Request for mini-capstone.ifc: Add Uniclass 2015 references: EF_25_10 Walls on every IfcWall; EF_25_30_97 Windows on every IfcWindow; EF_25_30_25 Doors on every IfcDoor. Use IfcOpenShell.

First a look at what the model holds.

```python
import ifcopenshell

model = ifcopenshell.open("mini-capstone.ifc")
print(model.schema)
print("classifications:", [c.Name for c in model.by_type("IfcClassification")])
for ifc_class in ("IfcDoor", "IfcRoof", "IfcStair", "IfcWall", "IfcWindow"):
    print(ifc_class, len(model.by_type(ifc_class)))
```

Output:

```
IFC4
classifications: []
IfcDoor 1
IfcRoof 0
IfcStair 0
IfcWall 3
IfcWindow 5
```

```python
import ifcopenshell
import ifcopenshell.api.classification

model = ifcopenshell.open("mini-capstone.ifc")

system = ifcopenshell.api.classification.add_classification(model, classification="Uniclass 2015")

codes = {
    "IfcWall": ("EF_25_10", "Walls"),
    "IfcWindow": ("EF_25_30_97", "Windows"),
    "IfcDoor": ("EF_25_30_25", "Doors"),
}
for ifc_class, (code, name) in codes.items():
    products = model.by_type(ifc_class)
    ifcopenshell.api.classification.add_reference(
        model, products=products, classification=system, identification=code, name=name
    )
    print(code, len(products))

model.write("mini-capstone_edited.ifc")
```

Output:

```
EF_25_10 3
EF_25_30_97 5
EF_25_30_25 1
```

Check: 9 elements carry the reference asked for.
